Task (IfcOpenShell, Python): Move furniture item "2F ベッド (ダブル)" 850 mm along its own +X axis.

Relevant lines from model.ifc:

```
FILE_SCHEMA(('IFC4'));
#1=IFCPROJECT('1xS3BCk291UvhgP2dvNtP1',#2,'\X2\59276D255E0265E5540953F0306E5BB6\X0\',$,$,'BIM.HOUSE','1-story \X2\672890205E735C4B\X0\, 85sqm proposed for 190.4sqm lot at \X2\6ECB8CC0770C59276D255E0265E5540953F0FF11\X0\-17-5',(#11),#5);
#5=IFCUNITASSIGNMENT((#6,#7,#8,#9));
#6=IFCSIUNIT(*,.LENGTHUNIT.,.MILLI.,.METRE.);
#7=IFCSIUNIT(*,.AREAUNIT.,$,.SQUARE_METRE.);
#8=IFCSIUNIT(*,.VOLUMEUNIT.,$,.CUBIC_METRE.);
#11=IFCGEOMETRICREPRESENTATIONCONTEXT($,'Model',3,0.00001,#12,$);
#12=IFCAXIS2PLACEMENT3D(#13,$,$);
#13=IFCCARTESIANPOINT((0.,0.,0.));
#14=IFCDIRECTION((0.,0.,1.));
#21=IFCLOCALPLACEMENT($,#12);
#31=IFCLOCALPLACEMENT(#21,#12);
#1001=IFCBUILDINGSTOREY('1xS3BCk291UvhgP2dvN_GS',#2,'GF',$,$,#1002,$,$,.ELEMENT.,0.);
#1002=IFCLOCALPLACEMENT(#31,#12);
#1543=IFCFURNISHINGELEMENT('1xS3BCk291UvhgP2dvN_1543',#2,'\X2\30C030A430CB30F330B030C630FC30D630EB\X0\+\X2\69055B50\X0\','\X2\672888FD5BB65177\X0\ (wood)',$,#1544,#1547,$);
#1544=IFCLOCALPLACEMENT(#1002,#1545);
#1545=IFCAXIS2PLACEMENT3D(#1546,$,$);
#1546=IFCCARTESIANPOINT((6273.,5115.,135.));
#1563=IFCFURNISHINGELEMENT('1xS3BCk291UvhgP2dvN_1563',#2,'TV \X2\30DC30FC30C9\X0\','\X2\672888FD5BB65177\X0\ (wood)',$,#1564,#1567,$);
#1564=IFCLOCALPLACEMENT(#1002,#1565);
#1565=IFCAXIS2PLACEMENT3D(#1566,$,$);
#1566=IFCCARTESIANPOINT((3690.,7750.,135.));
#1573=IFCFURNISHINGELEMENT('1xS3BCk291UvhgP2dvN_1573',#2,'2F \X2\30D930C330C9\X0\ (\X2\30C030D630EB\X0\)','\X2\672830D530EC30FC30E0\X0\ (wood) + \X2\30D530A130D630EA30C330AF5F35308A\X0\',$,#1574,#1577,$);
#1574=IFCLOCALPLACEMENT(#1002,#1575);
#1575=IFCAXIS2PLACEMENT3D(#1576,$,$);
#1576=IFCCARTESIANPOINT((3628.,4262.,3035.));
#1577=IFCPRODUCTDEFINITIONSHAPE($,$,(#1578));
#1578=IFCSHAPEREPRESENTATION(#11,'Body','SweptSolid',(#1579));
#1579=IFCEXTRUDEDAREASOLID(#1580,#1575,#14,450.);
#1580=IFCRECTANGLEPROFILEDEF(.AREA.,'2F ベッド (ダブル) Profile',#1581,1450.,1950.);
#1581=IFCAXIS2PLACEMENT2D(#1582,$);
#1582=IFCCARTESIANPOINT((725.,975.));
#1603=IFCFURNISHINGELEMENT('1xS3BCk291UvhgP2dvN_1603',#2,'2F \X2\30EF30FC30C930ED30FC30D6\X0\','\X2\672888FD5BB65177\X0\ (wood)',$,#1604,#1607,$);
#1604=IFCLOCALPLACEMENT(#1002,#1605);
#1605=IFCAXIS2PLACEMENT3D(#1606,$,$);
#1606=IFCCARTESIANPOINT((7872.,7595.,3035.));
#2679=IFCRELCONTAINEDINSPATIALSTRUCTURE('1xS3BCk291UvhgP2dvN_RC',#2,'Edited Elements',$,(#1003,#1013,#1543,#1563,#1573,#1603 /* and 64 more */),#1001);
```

```python
import ifcopenshell
import ifcopenshell.api.geometry
import ifcopenshell.util.placement

model = ifcopenshell.open("model.ifc")

item = model.by_guid("1xS3BCk291UvhgP2dvN_1573")
matrix = ifcopenshell.util.placement.get_local_placement(item.ObjectPlacement)
matrix[:3, 3] += matrix[:3, 0] * 850.0
ifcopenshell.api.geometry.edit_object_placement(model, product=item, matrix=matrix, is_si=False)

print(ifcopenshell.util.placement.get_local_placement(item.ObjectPlacement).round(3) + 0.0)

model.write("model_updated.ifc")
```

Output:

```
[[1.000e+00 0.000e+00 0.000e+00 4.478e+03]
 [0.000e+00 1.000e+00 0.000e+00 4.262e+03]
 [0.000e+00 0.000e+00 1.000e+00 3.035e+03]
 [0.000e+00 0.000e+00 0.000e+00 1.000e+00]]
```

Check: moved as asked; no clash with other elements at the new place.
